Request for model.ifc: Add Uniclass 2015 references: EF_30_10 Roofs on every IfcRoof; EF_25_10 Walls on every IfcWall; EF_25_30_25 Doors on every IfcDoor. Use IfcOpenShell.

First a look at what the model holds.

```python
import ifcopenshell

model = ifcopenshell.open("model.ifc")
print(model.schema)
print("classifications:", [c.Name for c in model.by_type("IfcClassification")])
for ifc_class in ("IfcDoor", "IfcRoof", "IfcStair", "IfcWall", "IfcWindow"):
    print(ifc_class, len(model.by_type(ifc_class)))
```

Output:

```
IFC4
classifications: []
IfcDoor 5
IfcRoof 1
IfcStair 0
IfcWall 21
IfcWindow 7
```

```python
import ifcopenshell
import ifcopenshell.api.classification

model = ifcopenshell.open("model.ifc")

system = ifcopenshell.api.classification.add_classification(model, classification="Uniclass 2015")

codes = {
    "IfcRoof": ("EF_30_10", "Roofs"),
    "IfcWall": ("EF_25_10", "Walls"),
    "IfcDoor": ("EF_25_30_25", "Doors"),
}
for ifc_class, (code, name) in codes.items():
    products = model.by_type(ifc_class)
    ifcopenshell.api.classification.add_reference(
        model, products=products, classification=system, identification=code, name=name
    )
    print(code, len(products))

model.write("model_v2.ifc")
```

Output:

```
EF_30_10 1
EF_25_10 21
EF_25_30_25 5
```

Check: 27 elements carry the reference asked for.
